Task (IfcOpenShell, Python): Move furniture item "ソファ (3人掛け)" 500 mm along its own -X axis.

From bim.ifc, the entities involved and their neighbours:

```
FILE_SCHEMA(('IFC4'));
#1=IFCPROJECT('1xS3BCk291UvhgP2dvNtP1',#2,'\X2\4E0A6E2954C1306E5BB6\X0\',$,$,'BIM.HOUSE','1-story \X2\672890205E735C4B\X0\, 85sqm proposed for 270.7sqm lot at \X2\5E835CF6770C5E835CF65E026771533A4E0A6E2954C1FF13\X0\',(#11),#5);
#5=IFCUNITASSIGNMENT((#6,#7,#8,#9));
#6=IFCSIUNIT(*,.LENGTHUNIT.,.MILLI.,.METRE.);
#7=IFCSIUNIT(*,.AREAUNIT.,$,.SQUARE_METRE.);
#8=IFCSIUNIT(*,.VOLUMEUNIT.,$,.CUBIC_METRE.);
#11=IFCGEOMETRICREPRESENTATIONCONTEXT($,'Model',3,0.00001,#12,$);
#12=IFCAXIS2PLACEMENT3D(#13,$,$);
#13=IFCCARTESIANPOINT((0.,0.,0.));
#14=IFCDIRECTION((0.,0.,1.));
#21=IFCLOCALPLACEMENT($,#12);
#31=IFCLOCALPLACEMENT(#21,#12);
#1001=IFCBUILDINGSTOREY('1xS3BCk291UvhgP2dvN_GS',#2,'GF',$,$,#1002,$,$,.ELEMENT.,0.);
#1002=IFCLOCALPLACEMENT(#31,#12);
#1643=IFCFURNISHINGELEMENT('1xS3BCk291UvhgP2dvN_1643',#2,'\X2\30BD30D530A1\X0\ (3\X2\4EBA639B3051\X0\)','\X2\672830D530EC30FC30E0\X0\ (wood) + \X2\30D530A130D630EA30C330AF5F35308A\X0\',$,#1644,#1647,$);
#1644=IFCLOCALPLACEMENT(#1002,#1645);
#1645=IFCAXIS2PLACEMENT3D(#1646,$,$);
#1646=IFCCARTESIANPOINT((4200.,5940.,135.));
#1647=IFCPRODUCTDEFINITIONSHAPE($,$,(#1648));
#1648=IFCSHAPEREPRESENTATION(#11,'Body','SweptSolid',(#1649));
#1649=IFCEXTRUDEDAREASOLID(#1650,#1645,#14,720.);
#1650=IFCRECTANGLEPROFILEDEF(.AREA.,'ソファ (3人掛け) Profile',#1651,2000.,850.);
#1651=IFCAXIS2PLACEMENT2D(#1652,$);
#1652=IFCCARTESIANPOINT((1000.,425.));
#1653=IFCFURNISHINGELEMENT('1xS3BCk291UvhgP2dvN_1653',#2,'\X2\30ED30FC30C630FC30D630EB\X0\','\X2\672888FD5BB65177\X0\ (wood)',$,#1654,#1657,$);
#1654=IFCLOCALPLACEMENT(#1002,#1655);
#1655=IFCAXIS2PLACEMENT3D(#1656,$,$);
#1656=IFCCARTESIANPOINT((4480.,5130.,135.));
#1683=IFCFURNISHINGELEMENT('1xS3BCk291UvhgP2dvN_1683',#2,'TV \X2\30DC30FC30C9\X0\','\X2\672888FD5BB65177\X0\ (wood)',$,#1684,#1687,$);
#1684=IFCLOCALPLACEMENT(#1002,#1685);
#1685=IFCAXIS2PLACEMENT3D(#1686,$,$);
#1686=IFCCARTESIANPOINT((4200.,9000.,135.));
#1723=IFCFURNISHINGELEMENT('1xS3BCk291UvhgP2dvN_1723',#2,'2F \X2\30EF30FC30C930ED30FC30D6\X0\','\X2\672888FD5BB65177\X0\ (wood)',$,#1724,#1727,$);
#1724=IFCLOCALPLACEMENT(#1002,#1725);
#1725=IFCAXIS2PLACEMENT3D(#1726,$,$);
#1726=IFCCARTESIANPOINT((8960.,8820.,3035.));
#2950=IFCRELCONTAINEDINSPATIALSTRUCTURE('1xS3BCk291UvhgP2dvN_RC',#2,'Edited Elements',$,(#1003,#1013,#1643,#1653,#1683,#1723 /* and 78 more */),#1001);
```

```python
import ifcopenshell
import ifcopenshell.api.geometry
import ifcopenshell.util.placement
import ifcopenshell.util.unit

model = ifcopenshell.open("bim.ifc")
unit_scale = ifcopenshell.util.unit.calculate_unit_scale(model)

item = model.by_guid("1xS3BCk291UvhgP2dvN_1643")
matrix = ifcopenshell.util.placement.get_local_placement(item.ObjectPlacement)
matrix[:3, 3] -= matrix[:3, 0] * 0.5 / unit_scale
ifcopenshell.api.geometry.edit_object_placement(model, product=item, matrix=matrix, is_si=False)

print(ifcopenshell.util.placement.get_local_placement(item.ObjectPlacement).round(3) + 0.0)

model.write("bim_rev.ifc")
```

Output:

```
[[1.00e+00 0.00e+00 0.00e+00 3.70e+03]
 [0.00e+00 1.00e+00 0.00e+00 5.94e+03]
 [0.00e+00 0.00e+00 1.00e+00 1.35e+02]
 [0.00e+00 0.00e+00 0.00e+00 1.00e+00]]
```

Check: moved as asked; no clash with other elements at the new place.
